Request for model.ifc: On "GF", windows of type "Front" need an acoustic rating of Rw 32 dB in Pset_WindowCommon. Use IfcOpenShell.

First a look at what the model holds.

```python
import ifcopenshell
import ifcopenshell.util.element

model = ifcopenshell.open("model.ifc")
print(model.schema)
storey = next(s for s in model.by_type("IfcBuildingStorey") if s.Name == "GF")
windows = [e for e in ifcopenshell.util.element.get_decomposition(storey) if e.is_a("IfcWindow")]
seen = {}
for e in windows:
    element_type = ifcopenshell.util.element.get_type(e)
    key = (element_type.Name if element_type != e and element_type else None, ifcopenshell.util.element.get_pset(e, "Pset_WindowCommon", "AcousticRating"))
    seen[key] = seen.get(key, 0) + 1
for (name, value), count in sorted(seen.items(), key=str):
    print(count, "x", name, "|", value)
```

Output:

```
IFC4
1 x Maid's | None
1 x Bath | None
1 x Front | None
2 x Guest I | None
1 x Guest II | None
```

```python
import ifcopenshell
import ifcopenshell.api.pset
import ifcopenshell.util.element

model = ifcopenshell.open("model.ifc")

storey = next(s for s in model.by_type("IfcBuildingStorey") if s.Name == "GF")
windows = [e for e in ifcopenshell.util.element.get_decomposition(storey) if e.is_a("IfcWindow")]

count = 0
for e in windows:
    element_type = ifcopenshell.util.element.get_type(e)
    if element_type in (None, e) or element_type.Name != "Front":
        continue
    # add_pset returns the element's existing set when there is one.
    pset = ifcopenshell.api.pset.add_pset(model, product=e, name="Pset_WindowCommon")
    ifcopenshell.api.pset.edit_pset(model, pset=pset, properties={"AcousticRating": "Rw 32 dB"})
    count += 1

print(count, "windows updated")

model.write("model_rev.ifc")
```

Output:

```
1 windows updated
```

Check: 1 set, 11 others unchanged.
